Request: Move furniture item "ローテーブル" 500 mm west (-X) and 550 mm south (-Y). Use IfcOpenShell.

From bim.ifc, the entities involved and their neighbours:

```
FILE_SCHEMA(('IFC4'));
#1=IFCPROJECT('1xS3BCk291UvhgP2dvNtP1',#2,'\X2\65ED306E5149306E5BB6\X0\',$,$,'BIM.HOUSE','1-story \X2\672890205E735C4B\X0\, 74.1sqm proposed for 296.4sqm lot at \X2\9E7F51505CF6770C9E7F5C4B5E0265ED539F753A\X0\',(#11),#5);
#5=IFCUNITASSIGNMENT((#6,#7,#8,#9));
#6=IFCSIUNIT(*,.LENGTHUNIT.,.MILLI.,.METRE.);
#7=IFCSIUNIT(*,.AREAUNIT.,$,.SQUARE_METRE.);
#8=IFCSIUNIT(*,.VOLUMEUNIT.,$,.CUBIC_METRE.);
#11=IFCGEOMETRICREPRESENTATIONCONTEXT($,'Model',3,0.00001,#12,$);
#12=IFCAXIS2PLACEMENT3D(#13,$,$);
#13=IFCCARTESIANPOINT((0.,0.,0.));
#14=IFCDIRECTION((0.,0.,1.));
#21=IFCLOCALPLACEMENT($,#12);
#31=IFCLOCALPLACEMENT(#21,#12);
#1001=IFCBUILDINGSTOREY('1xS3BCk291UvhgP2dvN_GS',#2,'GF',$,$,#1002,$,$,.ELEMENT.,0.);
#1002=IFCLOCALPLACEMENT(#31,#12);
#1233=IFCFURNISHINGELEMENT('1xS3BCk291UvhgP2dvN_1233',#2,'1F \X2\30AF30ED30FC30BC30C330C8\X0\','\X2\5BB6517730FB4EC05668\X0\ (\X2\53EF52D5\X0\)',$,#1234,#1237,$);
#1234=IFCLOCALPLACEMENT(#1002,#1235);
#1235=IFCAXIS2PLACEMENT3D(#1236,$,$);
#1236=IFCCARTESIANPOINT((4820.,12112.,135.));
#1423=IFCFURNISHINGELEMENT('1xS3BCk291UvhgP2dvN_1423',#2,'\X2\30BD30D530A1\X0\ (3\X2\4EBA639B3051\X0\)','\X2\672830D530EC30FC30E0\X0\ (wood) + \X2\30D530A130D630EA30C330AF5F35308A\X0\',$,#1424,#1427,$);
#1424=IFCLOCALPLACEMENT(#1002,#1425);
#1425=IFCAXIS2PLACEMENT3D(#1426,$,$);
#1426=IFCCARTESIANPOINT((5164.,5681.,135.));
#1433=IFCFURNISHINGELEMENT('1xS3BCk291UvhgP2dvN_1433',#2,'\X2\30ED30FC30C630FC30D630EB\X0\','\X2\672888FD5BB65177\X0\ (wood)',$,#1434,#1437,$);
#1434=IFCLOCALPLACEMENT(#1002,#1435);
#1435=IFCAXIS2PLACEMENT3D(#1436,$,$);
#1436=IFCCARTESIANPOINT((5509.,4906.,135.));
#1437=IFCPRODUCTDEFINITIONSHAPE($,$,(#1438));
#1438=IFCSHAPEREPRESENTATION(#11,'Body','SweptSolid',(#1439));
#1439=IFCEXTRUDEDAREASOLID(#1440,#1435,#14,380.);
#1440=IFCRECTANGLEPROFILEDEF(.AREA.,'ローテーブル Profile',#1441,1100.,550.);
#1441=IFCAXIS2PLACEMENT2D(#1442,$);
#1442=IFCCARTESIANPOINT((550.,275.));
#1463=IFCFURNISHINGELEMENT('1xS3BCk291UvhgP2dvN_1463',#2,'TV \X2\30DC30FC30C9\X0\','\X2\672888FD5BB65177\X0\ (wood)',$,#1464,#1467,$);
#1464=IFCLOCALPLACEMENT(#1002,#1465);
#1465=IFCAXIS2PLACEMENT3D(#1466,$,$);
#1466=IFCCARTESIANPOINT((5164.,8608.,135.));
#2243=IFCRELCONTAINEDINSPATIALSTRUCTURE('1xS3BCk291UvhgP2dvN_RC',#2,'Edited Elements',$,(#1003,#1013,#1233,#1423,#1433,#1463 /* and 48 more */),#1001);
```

```python
import ifcopenshell
import ifcopenshell.api.geometry
import ifcopenshell.util.placement
import ifcopenshell.util.unit

model = ifcopenshell.open("bim.ifc")
unit_scale = ifcopenshell.util.unit.calculate_unit_scale(model)

item = model.by_guid("1xS3BCk291UvhgP2dvN_1433")
matrix = ifcopenshell.util.placement.get_local_placement(item.ObjectPlacement)
matrix[0, 3] -= 0.5 / unit_scale
matrix[1, 3] -= 0.55 / unit_scale
ifcopenshell.api.geometry.edit_object_placement(model, product=item, matrix=matrix, is_si=False)

print(ifcopenshell.util.placement.get_local_placement(item.ObjectPlacement).round(3) + 0.0)

model.write("bim-out.ifc")
```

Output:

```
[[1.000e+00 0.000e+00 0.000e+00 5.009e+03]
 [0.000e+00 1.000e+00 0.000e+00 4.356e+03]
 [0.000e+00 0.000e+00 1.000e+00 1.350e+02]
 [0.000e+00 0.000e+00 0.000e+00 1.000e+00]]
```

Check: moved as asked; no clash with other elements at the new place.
